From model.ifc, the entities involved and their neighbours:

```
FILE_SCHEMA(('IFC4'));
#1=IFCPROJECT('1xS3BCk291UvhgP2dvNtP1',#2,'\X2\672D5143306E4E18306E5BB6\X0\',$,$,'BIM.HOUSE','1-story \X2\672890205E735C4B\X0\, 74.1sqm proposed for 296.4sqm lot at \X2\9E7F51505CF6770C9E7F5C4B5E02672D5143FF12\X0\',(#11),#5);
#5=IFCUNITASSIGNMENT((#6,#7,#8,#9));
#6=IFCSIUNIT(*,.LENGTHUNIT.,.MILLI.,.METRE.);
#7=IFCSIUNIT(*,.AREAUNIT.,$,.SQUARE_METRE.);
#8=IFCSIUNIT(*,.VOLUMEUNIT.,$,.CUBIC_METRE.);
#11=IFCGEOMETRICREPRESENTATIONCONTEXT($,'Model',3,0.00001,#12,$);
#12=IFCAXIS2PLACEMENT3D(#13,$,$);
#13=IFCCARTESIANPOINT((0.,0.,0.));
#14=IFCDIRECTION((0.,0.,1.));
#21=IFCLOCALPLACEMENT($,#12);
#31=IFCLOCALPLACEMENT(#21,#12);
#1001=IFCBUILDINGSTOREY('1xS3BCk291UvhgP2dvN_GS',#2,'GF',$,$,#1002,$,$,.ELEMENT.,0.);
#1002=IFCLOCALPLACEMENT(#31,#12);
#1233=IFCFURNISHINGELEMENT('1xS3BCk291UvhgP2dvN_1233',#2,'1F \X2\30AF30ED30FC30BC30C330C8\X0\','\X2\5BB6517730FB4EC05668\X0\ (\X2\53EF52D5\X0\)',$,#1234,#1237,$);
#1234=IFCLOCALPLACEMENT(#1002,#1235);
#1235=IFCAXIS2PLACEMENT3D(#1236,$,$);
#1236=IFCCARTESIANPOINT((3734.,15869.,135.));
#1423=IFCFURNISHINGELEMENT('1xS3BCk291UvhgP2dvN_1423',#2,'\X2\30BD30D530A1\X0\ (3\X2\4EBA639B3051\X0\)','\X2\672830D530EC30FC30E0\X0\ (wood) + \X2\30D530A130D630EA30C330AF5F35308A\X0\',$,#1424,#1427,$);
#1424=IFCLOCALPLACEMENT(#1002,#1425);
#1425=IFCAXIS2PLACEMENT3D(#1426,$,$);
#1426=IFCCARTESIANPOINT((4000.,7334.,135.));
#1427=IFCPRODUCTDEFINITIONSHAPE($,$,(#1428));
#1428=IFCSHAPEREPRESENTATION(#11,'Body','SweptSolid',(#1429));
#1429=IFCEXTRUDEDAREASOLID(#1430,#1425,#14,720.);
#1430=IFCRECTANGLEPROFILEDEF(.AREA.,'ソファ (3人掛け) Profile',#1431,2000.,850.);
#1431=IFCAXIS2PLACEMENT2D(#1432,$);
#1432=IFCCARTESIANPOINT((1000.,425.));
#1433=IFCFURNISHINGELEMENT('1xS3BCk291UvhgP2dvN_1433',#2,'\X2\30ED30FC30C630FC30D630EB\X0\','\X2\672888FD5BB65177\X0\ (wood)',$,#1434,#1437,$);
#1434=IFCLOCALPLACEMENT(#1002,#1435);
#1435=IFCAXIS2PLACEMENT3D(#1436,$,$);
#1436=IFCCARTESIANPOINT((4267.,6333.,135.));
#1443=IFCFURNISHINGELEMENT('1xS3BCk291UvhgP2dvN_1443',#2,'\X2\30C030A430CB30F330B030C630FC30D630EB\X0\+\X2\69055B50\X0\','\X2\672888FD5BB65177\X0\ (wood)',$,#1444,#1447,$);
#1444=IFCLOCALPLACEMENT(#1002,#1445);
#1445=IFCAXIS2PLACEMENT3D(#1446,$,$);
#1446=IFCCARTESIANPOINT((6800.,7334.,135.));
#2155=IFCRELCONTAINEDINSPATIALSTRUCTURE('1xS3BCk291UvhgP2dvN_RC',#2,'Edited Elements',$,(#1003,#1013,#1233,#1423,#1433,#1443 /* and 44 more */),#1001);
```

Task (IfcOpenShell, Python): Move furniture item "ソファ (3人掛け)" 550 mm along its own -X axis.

```python
import ifcopenshell
import ifcopenshell.api.geometry
import ifcopenshell.util.placement
import ifcopenshell.util.unit

model = ifcopenshell.open("model.ifc")
unit_scale = ifcopenshell.util.unit.calculate_unit_scale(model)

item = model.by_id(1423)
matrix = ifcopenshell.util.placement.get_local_placement(item.ObjectPlacement)
matrix[:3, 3] -= matrix[:3, 0] * 0.55 / unit_scale
ifcopenshell.api.geometry.edit_object_placement(model, product=item, matrix=matrix, is_si=False)

print(ifcopenshell.util.placement.get_local_placement(item.ObjectPlacement).round(3) + 0.0)

model.write("model_updated.ifc")
```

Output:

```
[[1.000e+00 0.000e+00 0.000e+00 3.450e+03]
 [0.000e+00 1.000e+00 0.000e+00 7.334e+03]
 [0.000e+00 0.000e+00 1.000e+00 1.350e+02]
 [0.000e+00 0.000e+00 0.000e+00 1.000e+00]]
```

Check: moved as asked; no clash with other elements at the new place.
